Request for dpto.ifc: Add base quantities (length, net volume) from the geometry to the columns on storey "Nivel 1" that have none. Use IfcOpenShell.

First a look at what the model holds.

```python
import ifcopenshell
import ifcopenshell.util.element
import ifcopenshell.util.unit

model = ifcopenshell.open("dpto.ifc")
print(model.schema)
for unit_type in ("LENGTHUNIT", "AREAUNIT", "VOLUMEUNIT"):
    print(unit_type, ifcopenshell.util.unit.calculate_unit_scale(model, unit_type))
storey = next(s for s in model.by_type("IfcBuildingStorey") if s.Name == "Nivel 1")
columns = [e for e in ifcopenshell.util.element.get_decomposition(storey) if e.is_a("IfcColumn")]
for e in sorted(columns, key=lambda e: e.id()):
    print(e.id(), e.is_a(), e.Name, list(ifcopenshell.util.element.get_psets(e, qtos_only=True)), sep=" | ")
```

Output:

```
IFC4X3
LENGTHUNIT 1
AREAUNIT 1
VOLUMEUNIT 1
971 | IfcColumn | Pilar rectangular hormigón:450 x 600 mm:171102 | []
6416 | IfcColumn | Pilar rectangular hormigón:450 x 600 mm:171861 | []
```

```python
import ifcopenshell
import ifcopenshell.api.pset
import ifcopenshell.geom
import ifcopenshell.util.element
import ifcopenshell.util.shape
import ifcopenshell.util.unit

model = ifcopenshell.open("dpto.ifc")
unit_scale = ifcopenshell.util.unit.calculate_unit_scale(model)
volume_scale = ifcopenshell.util.unit.calculate_unit_scale(model, "VOLUMEUNIT")
settings = ifcopenshell.geom.settings()

storey = next(s for s in model.by_type("IfcBuildingStorey") if s.Name == "Nivel 1")
columns = [e for e in ifcopenshell.util.element.get_decomposition(storey) if e.is_a("IfcColumn")]

for e in sorted(columns, key=lambda e: e.id()):
    if ifcopenshell.util.element.get_psets(e, qtos_only=True, should_inherit=False):
        continue
    # Geometry comes back in metres, in the element's own axes.
    shape = ifcopenshell.geom.create_shape(settings, e)
    values = {
        "Length": ifcopenshell.util.shape.get_z(shape.geometry) / unit_scale,
        "NetVolume": ifcopenshell.util.shape.get_volume(shape.geometry) / volume_scale,
    }
    qto = ifcopenshell.api.pset.add_qto(model, product=e, name="Qto_ColumnBaseQuantities")
    ifcopenshell.api.pset.edit_qto(model, qto=qto, properties=values)
    print(e.id(), {k: round(v, 3) for k, v in values.items()})

model.write("dpto_edited.ifc")
```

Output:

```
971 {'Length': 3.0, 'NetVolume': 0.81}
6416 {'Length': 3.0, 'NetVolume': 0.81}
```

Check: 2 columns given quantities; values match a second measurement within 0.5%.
